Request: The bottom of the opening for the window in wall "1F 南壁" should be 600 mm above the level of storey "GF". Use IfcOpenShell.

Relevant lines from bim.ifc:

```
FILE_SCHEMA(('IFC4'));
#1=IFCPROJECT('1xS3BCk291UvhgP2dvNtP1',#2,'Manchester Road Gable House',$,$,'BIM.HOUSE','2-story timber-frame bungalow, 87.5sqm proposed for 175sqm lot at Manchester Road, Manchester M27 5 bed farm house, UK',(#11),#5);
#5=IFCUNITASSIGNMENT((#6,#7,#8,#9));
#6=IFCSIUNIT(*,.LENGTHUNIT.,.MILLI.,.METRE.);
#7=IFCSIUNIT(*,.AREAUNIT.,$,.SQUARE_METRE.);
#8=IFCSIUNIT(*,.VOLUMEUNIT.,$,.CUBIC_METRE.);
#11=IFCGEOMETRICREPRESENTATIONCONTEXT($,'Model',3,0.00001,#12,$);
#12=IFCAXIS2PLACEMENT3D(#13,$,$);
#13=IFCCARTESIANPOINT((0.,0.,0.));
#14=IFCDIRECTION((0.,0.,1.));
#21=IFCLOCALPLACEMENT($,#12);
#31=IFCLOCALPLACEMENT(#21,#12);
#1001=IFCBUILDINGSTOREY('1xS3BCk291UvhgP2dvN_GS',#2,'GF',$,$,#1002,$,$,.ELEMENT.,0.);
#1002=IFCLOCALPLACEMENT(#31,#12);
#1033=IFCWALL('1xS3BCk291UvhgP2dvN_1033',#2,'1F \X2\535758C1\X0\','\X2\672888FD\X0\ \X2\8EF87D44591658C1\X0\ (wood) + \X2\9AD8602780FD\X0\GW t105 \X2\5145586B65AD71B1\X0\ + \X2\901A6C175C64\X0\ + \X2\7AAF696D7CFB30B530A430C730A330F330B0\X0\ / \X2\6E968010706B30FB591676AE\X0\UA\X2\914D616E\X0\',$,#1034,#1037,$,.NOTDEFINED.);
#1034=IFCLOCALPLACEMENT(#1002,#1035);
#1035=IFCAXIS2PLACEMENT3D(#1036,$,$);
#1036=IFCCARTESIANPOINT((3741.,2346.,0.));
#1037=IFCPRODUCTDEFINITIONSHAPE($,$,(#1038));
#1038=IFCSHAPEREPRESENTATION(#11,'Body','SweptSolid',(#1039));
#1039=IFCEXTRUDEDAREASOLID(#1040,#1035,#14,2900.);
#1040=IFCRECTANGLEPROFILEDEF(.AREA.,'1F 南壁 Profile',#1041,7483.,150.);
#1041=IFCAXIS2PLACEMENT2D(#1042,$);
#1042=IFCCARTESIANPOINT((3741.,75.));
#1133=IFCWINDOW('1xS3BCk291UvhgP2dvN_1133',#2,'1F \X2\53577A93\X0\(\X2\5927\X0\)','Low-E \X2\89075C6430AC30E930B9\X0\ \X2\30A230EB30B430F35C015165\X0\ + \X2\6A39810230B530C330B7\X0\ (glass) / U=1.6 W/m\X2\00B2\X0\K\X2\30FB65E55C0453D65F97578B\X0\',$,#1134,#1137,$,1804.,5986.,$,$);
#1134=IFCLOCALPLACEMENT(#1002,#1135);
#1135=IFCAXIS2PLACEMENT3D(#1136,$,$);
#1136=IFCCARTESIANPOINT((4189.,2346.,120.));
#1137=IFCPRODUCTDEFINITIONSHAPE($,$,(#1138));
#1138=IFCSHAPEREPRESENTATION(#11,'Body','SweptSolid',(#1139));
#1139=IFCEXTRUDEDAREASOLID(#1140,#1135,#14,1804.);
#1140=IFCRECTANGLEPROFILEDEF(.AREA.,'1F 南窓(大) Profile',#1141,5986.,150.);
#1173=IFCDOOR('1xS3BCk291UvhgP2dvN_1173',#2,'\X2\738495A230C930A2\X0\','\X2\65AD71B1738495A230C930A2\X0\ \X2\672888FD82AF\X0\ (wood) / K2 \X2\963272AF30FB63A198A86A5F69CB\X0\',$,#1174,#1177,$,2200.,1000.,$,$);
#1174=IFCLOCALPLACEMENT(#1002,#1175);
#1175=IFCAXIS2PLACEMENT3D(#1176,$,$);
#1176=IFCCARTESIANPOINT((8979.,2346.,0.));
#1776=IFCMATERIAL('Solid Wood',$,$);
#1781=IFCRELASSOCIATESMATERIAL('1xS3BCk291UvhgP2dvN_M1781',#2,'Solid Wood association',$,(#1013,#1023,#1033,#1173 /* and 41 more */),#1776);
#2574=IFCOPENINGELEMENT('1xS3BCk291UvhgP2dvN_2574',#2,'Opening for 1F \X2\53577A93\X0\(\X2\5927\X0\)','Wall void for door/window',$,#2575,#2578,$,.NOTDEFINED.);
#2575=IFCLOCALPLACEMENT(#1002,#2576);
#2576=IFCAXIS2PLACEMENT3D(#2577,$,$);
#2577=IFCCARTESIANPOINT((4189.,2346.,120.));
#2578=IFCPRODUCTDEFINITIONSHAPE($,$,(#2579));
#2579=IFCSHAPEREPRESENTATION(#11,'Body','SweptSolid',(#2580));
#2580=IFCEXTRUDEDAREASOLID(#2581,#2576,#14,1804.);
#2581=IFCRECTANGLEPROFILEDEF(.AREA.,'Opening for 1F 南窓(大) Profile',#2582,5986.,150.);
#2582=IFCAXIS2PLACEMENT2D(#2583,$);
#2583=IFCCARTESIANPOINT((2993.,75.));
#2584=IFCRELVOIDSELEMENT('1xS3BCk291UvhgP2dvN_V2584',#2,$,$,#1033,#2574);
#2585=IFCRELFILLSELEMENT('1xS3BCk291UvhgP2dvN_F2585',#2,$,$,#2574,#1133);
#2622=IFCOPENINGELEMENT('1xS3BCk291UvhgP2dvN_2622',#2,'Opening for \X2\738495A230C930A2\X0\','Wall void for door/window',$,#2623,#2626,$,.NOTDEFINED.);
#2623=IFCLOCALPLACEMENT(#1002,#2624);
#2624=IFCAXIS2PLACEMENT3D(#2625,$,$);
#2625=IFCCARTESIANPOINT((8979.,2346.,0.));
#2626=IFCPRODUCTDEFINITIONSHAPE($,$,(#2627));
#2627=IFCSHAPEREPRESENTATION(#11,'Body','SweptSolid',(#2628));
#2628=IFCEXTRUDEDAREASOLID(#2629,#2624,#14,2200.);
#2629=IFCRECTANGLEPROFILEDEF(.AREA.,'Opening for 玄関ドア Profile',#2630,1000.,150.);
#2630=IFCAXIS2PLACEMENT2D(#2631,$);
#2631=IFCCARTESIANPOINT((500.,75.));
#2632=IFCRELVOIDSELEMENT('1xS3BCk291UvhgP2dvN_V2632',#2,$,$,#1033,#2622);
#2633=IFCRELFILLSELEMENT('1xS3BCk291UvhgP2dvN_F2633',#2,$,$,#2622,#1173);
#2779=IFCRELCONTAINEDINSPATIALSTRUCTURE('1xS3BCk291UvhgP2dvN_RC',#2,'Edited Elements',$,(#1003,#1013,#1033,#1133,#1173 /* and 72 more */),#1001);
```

```python
import numpy as np
import ifcopenshell
import ifcopenshell.api.geometry
import ifcopenshell.geom
import ifcopenshell.util.element
import ifcopenshell.util.placement
import ifcopenshell.util.shape
import ifcopenshell.util.unit

model = ifcopenshell.open("bim.ifc")
unit_scale = ifcopenshell.util.unit.calculate_unit_scale(model)

window = model.by_id(1133)
opening = window.FillsVoids[0].RelatingOpeningElement
storey = ifcopenshell.util.element.get_container(window, ifc_class="IfcBuildingStorey")
level = ifcopenshell.util.placement.get_local_placement(storey.ObjectPlacement)[2, 3]

# The opening's origin need not be at the sill, so measure its lowest point.
shape = ifcopenshell.geom.create_shape(ifcopenshell.geom.settings(), opening)
bottom = ifcopenshell.util.shape.get_shape_bottom_elevation(shape, shape.geometry) / unit_scale
dz = level + 600.0 - bottom

shift = np.array([0.0, 0.0, dz])
# The window is not placed relative to its opening, so move both.
for product in (opening, window):
    matrix = ifcopenshell.util.placement.get_local_placement(product.ObjectPlacement)
    matrix[:3, 3] += shift
    ifcopenshell.api.geometry.edit_object_placement(model, product=product, matrix=matrix, is_si=False)

print(f"moved by {dz * unit_scale:+.3f} m")

model.write("bim_updated.ifc")
```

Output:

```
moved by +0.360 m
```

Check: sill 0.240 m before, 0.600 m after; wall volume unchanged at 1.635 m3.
